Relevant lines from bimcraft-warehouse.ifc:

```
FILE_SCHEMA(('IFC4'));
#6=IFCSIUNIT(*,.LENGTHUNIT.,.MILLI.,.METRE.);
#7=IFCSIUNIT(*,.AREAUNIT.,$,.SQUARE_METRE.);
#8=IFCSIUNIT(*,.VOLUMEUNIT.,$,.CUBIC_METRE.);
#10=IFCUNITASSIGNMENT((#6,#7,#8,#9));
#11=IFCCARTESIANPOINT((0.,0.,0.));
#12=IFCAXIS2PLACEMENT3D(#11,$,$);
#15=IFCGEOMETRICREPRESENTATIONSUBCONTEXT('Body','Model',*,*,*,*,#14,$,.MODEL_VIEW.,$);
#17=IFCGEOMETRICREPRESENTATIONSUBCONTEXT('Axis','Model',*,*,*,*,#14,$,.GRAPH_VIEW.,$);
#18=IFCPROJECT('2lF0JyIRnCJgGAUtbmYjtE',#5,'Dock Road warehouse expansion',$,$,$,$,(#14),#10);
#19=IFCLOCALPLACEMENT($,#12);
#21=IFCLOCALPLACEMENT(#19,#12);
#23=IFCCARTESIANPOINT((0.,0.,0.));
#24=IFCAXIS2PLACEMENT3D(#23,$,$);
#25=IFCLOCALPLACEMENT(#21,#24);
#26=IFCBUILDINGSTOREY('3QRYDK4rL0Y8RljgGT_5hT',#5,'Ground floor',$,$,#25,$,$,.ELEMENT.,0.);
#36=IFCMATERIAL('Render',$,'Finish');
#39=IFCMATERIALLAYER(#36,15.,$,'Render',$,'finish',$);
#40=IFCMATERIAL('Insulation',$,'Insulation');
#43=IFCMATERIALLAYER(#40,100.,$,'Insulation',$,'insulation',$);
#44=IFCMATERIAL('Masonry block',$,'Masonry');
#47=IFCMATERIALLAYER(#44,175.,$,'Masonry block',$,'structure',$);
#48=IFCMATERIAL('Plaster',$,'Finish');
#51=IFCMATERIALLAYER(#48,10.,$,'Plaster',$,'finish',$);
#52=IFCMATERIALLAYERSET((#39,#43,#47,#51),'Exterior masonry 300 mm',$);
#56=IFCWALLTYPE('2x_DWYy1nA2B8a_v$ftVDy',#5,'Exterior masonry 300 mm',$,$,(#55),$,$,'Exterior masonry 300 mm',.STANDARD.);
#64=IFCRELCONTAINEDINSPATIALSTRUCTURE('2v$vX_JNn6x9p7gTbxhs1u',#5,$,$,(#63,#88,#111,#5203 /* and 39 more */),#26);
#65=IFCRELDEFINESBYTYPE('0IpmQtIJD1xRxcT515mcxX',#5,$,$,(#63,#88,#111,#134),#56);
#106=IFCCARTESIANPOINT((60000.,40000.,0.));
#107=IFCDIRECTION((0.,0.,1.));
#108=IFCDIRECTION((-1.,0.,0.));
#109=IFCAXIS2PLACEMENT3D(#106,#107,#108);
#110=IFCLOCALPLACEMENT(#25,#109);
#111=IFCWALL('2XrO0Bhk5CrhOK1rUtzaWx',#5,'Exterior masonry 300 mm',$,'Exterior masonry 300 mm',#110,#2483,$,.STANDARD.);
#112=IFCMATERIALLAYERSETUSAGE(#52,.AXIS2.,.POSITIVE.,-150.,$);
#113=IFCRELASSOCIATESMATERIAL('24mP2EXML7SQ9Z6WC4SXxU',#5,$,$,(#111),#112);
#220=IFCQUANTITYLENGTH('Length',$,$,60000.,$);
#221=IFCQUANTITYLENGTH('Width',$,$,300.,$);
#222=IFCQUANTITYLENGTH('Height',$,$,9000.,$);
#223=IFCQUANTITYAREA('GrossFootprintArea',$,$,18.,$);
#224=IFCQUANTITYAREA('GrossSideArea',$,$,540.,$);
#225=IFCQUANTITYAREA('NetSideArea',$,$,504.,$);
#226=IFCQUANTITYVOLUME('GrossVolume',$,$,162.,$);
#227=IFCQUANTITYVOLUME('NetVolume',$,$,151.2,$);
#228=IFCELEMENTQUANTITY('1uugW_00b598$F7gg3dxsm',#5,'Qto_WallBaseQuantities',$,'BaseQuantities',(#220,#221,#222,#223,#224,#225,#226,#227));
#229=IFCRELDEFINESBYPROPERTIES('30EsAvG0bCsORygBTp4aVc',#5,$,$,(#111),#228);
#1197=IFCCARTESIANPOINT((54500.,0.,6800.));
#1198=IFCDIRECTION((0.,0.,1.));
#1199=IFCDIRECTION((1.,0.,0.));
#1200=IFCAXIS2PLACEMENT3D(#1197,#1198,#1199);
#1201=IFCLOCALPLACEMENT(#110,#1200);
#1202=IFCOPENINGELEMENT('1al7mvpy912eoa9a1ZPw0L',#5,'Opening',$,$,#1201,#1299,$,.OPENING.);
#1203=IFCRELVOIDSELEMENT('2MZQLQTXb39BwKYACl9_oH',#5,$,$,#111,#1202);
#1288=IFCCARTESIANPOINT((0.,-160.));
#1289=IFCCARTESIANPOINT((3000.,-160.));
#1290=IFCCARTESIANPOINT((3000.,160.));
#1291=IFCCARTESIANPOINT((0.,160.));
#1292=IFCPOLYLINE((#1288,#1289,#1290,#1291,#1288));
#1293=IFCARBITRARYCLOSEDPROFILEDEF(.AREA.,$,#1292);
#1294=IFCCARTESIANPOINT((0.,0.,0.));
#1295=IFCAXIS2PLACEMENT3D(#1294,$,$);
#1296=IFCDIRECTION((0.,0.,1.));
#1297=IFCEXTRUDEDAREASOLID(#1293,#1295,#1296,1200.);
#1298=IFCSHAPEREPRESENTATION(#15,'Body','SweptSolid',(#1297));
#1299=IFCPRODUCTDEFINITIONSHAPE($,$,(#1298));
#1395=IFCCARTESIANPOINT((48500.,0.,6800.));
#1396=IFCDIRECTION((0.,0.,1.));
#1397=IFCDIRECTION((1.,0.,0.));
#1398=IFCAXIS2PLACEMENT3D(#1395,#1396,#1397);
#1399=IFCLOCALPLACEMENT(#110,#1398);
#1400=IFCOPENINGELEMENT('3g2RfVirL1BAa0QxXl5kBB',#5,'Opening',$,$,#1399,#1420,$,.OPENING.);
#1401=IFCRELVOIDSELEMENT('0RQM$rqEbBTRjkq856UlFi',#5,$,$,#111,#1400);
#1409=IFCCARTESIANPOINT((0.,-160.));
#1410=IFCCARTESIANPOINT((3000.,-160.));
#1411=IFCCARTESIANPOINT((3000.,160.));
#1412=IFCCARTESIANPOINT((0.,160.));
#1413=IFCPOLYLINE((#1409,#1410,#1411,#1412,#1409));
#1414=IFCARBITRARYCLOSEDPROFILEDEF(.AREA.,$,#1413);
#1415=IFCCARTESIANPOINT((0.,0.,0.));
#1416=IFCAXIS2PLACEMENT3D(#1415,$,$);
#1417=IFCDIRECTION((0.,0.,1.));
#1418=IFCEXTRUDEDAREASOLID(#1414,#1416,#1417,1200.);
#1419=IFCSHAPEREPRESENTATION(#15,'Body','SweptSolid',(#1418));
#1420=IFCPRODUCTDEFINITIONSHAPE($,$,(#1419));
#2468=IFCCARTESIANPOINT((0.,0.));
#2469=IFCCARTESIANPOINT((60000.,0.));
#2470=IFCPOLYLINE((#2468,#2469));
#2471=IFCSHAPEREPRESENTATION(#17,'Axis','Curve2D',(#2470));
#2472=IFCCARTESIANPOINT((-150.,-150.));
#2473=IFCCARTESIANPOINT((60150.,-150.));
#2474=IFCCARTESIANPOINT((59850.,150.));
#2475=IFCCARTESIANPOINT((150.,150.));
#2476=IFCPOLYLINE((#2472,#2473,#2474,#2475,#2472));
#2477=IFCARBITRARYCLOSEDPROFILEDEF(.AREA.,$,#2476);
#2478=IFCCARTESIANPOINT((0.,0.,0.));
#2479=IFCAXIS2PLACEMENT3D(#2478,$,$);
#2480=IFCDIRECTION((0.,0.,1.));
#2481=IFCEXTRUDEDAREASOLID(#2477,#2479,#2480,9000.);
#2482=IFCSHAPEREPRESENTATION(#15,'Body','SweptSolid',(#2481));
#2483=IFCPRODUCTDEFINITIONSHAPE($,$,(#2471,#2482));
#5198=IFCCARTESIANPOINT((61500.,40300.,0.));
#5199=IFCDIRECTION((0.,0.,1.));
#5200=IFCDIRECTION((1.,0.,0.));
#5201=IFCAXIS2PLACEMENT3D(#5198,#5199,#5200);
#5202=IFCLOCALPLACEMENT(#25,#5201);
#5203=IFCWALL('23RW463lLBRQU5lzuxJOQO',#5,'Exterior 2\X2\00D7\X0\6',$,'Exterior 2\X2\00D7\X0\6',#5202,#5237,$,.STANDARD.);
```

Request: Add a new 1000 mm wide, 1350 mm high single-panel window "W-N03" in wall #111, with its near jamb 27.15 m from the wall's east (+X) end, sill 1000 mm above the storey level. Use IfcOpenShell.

```python
import numpy as np
import ifcopenshell
import ifcopenshell.api.feature
import ifcopenshell.api.geometry
import ifcopenshell.api.pset
import ifcopenshell.api.root
import ifcopenshell.api.spatial
import ifcopenshell.geom
import ifcopenshell.util.element
import ifcopenshell.util.placement
import ifcopenshell.util.representation
import ifcopenshell.util.shape
import ifcopenshell.util.unit

model = ifcopenshell.open("bimcraft-warehouse.ifc")
unit_scale = ifcopenshell.util.unit.calculate_unit_scale(model)
area_scale = ifcopenshell.util.unit.calculate_unit_scale(model, "AREAUNIT")
volume_scale = ifcopenshell.util.unit.calculate_unit_scale(model, "VOLUMEUNIT")
settings = ifcopenshell.geom.settings()


def volume(element):
    """Net volume in cubic metres, openings subtracted."""
    shape = ifcopenshell.geom.create_shape(settings, element)
    return ifcopenshell.util.shape.get_volume(shape.geometry)


wall = model.by_guid("2XrO0Bhk5CrhOK1rUtzaWx")
storey = ifcopenshell.util.element.get_container(wall, ifc_class="IfcBuildingStorey")
context = ifcopenshell.util.representation.get_context(model, "Model", "Body", "MODEL_VIEW")
before = volume(wall)

width, height, from_end, sill = 1, 1.35, 27.15, 1  # metres

# The wall runs along its own X axis, and the end named is its -X end.
wall_shape = ifcopenshell.geom.create_shape(settings, wall)
x, y, z = ifcopenshell.util.shape.get_vertices(wall_shape.geometry).T
start = x.min() + from_end
face, thickness = float(y.min()), float(y.max() - y.min())
wall_matrix = ifcopenshell.util.placement.get_local_placement(wall.ObjectPlacement)
level = ifcopenshell.util.placement.get_local_placement(storey.ObjectPlacement)[2, 3]


def in_wall(x, y):
    """Placement at x, y metres in the wall's axes, at sill height."""
    matrix = wall_matrix.copy()
    matrix[:, 3] = wall_matrix @ np.array([x / unit_scale, y / unit_scale, 0.0, 1.0])
    matrix[2, 3] = level + sill / unit_scale
    return matrix


# Opening: a box that overshoots both wall faces by 50 mm.
opening = ifcopenshell.api.root.create_entity(model, ifc_class="IfcOpeningElement", predefined_type="OPENING")
box = ifcopenshell.api.geometry.add_wall_representation(
    model, context=context, length=width, height=height, thickness=thickness + 0.1
)
ifcopenshell.api.geometry.assign_representation(model, product=opening, representation=box)
ifcopenshell.api.geometry.edit_object_placement(model, product=opening, matrix=in_wall(start, face - 0.05), is_si=False)
ifcopenshell.api.feature.add_feature(model, feature=opening, element=wall)

window = ifcopenshell.api.root.create_entity(model, ifc_class="IfcWindow", name="W-N03", predefined_type="WINDOW")
window.OverallWidth, window.OverallHeight = width / unit_scale, height / unit_scale
window.PartitioningType = "SINGLE_PANEL"
body = ifcopenshell.api.geometry.add_window_representation(
    model,
    context=context,
    overall_width=window.OverallWidth,
    overall_height=window.OverallHeight,
    partition_type="SINGLE_PANEL",
)
ifcopenshell.api.geometry.assign_representation(model, product=window, representation=body)
ifcopenshell.api.spatial.assign_container(model, products=[window], relating_structure=storey)
ifcopenshell.api.feature.add_filling(model, opening=opening, element=window)

# Centre the window in the wall's thickness.
ifcopenshell.api.geometry.edit_object_placement(model, product=window, matrix=in_wall(start, face), is_si=False)
window_shape = ifcopenshell.geom.create_shape(settings, window)
depth = ifcopenshell.util.shape.get_vertices(window_shape.geometry)[:, 1]
offset = face + thickness / 2 - (depth.min() + depth.max()) / 2
ifcopenshell.api.geometry.edit_object_placement(model, product=window, matrix=in_wall(start, offset), is_si=False)

after = volume(wall)

# Update the wall's stored quantities.
qto = model.by_id(ifcopenshell.util.element.get_pset(wall, "Qto_WallBaseQuantities", should_inherit=False)["id"])
ifcopenshell.api.pset.edit_qto(model, qto=qto, properties={
    "NetSideArea": after / thickness / area_scale,
    "NetVolume": after / volume_scale,
})

print(f"wall volume {before:.3f} -> {after:.3f} m3")

model.write("bimcraft-warehouse_edited.ifc")
```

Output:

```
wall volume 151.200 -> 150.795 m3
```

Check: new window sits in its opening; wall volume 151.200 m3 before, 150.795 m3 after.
